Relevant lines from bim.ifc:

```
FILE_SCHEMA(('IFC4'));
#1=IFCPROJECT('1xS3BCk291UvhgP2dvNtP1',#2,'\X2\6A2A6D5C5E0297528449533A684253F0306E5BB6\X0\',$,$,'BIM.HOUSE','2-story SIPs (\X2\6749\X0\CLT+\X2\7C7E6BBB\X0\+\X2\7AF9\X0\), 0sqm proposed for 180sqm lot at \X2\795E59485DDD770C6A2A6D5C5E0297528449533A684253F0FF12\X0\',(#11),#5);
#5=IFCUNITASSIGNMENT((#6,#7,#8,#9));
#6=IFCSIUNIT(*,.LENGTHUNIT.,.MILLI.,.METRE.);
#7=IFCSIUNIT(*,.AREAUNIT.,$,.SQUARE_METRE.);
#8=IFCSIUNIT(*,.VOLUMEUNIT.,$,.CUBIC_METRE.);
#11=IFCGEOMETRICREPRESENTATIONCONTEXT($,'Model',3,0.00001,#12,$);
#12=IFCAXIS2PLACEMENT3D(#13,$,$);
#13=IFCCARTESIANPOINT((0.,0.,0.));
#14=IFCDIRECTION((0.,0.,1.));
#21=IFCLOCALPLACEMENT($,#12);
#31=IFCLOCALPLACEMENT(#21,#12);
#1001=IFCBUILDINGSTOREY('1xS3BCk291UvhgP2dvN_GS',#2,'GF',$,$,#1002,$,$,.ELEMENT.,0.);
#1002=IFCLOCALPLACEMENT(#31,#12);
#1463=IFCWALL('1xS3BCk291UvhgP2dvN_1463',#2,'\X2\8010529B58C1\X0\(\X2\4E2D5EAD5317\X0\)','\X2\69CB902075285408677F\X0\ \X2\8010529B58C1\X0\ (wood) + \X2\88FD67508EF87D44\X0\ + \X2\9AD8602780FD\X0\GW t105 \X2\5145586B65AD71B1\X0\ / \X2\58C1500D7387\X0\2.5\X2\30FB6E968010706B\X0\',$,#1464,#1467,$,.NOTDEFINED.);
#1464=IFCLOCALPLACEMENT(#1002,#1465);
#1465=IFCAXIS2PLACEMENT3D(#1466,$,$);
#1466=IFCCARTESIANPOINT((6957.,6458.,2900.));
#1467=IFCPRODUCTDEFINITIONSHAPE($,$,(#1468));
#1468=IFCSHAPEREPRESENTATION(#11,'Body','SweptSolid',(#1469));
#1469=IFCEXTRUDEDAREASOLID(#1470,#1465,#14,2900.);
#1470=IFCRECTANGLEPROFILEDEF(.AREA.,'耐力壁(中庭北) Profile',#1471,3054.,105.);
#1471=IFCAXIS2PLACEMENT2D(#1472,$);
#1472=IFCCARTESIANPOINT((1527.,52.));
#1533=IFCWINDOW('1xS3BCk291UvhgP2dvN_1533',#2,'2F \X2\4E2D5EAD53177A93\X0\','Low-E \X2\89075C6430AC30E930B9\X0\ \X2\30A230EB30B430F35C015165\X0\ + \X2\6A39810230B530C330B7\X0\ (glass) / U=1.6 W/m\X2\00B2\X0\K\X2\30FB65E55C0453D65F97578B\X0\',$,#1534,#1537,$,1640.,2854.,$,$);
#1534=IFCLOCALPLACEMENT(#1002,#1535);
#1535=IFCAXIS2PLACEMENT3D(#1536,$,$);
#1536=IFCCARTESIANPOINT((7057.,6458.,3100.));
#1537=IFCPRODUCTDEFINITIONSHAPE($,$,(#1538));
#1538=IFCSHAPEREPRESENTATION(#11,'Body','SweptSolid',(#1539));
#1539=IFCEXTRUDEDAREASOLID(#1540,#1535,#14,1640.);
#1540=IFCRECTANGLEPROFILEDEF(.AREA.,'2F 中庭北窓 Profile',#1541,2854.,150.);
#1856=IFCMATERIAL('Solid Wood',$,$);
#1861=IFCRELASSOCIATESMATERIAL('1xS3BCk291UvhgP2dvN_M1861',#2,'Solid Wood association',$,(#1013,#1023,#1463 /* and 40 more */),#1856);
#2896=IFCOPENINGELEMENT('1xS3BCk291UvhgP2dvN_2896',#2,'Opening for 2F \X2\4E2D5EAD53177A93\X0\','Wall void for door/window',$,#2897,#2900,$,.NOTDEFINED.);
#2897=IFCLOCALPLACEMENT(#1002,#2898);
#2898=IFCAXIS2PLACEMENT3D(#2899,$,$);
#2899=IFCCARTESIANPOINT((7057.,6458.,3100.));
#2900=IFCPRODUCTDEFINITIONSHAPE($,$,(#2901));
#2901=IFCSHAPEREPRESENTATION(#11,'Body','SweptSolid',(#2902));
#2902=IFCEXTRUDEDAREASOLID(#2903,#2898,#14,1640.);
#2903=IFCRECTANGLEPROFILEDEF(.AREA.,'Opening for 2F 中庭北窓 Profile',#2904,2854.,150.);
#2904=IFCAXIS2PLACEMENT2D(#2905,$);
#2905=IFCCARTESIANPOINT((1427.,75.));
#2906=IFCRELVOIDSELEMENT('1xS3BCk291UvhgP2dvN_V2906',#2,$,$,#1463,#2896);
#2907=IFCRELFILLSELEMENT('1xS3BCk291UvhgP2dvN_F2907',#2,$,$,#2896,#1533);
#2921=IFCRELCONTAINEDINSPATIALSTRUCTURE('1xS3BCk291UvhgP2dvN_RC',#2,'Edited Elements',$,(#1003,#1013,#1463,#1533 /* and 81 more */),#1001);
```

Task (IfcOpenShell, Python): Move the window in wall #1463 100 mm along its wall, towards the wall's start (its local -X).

```python
import ifcopenshell
import ifcopenshell.api.geometry
import ifcopenshell.util.placement
import ifcopenshell.util.unit

model = ifcopenshell.open("bim.ifc")
unit_scale = ifcopenshell.util.unit.calculate_unit_scale(model)

window = model.by_id(1533)
opening = window.FillsVoids[0].RelatingOpeningElement
wall = opening.VoidsElements[0].RelatingBuildingElement

wall_matrix = ifcopenshell.util.placement.get_local_placement(wall.ObjectPlacement)
shift = wall_matrix[:3, 0] * -0.1 / unit_scale
before = ifcopenshell.util.placement.get_local_placement(window.ObjectPlacement)[:3, 3].copy()

# The window is not placed relative to its opening, so move both.
for product in (opening, window):
    matrix = ifcopenshell.util.placement.get_local_placement(product.ObjectPlacement)
    matrix[:3, 3] += shift
    ifcopenshell.api.geometry.edit_object_placement(model, product=product, matrix=matrix, is_si=False)

after = ifcopenshell.util.placement.get_local_placement(window.ObjectPlacement)[:3, 3]
print("window moved by", (after - before).round(3) + 0.0)

model.write("bim_rev.ifc")
```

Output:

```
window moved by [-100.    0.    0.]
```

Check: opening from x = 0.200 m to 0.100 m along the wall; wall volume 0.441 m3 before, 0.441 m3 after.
